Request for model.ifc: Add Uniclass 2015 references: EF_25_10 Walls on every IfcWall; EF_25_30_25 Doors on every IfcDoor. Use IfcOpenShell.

First a look at what the model holds.

```python
import ifcopenshell

model = ifcopenshell.open("model.ifc")
print(model.schema)
print("classifications:", [c.Name for c in model.by_type("IfcClassification")])
for ifc_class in ("IfcDoor", "IfcRoof", "IfcStair", "IfcWall", "IfcWindow"):
    print(ifc_class, len(model.by_type(ifc_class)))
```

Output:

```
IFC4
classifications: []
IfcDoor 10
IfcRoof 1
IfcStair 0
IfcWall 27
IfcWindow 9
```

```python
import ifcopenshell
import ifcopenshell.api.classification

model = ifcopenshell.open("model.ifc")

system = ifcopenshell.api.classification.add_classification(model, classification="Uniclass 2015")

codes = {
    "IfcWall": ("EF_25_10", "Walls"),
    "IfcDoor": ("EF_25_30_25", "Doors"),
}
for ifc_class, (code, name) in codes.items():
    products = model.by_type(ifc_class)
    ifcopenshell.api.classification.add_reference(
        model, products=products, classification=system, identification=code, name=name
    )
    print(code, len(products))

model.write("model_v2.ifc")
```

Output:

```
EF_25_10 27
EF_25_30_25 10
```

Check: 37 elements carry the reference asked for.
